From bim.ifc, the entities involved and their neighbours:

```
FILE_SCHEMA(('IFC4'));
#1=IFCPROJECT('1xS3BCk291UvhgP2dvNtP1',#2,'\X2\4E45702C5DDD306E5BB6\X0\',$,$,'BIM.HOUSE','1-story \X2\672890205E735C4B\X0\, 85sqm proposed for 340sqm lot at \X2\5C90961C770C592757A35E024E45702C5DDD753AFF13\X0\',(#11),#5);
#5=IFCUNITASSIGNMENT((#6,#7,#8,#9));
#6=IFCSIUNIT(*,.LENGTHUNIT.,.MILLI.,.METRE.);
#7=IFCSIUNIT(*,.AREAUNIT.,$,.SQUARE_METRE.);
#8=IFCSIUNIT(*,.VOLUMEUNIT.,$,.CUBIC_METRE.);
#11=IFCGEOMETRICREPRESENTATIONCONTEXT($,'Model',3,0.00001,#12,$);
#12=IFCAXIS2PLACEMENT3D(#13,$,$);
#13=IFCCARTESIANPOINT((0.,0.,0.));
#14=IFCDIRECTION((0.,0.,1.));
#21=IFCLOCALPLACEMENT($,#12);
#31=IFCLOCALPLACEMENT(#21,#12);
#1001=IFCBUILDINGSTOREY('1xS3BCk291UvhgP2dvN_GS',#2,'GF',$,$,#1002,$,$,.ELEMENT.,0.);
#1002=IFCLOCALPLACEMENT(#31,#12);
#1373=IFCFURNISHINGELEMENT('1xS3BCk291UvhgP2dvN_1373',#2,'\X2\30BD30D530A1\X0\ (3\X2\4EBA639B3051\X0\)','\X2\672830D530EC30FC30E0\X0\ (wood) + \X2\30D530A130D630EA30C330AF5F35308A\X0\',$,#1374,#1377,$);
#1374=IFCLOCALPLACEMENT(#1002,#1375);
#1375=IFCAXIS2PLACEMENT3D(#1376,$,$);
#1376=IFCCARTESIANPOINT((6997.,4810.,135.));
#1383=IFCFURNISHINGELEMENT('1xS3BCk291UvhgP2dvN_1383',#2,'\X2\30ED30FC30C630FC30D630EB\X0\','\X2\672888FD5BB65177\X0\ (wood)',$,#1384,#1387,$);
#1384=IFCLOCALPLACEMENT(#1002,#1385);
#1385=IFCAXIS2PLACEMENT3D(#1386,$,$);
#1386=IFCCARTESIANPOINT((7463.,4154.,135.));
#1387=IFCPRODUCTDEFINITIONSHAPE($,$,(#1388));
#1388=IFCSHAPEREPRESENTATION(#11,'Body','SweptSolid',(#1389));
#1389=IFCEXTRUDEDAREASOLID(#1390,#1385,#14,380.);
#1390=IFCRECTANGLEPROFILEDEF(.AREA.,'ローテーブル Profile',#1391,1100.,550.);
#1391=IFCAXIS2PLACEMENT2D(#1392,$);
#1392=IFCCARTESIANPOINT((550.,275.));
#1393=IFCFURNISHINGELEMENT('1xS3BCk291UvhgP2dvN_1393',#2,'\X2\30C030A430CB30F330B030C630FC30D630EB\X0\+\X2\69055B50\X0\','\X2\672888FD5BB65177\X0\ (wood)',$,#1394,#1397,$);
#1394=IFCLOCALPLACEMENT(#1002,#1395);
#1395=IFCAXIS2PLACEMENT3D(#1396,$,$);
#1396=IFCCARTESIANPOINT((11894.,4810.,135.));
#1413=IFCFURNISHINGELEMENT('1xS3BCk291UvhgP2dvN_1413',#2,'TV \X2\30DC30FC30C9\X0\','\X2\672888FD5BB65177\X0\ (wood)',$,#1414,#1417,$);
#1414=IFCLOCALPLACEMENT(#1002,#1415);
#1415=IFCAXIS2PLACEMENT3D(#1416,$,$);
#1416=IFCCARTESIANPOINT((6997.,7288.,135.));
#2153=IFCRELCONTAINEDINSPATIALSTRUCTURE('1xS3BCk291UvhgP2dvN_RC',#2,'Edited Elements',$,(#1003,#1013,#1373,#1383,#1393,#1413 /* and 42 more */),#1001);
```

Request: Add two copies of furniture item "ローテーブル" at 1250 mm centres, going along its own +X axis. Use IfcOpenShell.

```python
import ifcopenshell
import ifcopenshell.api.geometry
import ifcopenshell.api.root
import ifcopenshell.util.element
import ifcopenshell.util.placement
import ifcopenshell.util.unit

model = ifcopenshell.open("bim.ifc")
unit_scale = ifcopenshell.util.unit.calculate_unit_scale(model)


def reuse_history(source, copy):
    """copy_class also copies each property set's owner history, people and application; keep the originals."""
    for rel in copy.IsDefinedBy:
        if rel.is_a("IfcRelDefinesByProperties") and (history := rel.RelatingPropertyDefinition.OwnerHistory):
            rel.RelatingPropertyDefinition.OwnerHistory = source.OwnerHistory
            ifcopenshell.util.element.remove_deep2(model, history)


source = model.by_guid("1xS3BCk291UvhgP2dvN_1383")
base = ifcopenshell.util.placement.get_local_placement(source.ObjectPlacement)
step = base[:3, 0] * 1.25 / unit_scale

for i in range(1, 3):
    copy = ifcopenshell.api.root.copy_class(model, product=source)
    copy.Representation = ifcopenshell.util.element.copy_deep(
        model, source.Representation, exclude=["IfcGeometricRepresentationContext", "IfcRepresentationMap"]
    )
    reuse_history(source, copy)
    matrix = base.copy()
    matrix[:3, 3] += i * step
    print("added at", matrix[:3, 3].round(3) + 0.0)
    ifcopenshell.api.geometry.edit_object_placement(model, product=copy, matrix=matrix, is_si=False)

model.write("bim_rev.ifc")
```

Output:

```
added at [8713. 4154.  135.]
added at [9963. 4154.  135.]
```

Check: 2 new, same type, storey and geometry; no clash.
